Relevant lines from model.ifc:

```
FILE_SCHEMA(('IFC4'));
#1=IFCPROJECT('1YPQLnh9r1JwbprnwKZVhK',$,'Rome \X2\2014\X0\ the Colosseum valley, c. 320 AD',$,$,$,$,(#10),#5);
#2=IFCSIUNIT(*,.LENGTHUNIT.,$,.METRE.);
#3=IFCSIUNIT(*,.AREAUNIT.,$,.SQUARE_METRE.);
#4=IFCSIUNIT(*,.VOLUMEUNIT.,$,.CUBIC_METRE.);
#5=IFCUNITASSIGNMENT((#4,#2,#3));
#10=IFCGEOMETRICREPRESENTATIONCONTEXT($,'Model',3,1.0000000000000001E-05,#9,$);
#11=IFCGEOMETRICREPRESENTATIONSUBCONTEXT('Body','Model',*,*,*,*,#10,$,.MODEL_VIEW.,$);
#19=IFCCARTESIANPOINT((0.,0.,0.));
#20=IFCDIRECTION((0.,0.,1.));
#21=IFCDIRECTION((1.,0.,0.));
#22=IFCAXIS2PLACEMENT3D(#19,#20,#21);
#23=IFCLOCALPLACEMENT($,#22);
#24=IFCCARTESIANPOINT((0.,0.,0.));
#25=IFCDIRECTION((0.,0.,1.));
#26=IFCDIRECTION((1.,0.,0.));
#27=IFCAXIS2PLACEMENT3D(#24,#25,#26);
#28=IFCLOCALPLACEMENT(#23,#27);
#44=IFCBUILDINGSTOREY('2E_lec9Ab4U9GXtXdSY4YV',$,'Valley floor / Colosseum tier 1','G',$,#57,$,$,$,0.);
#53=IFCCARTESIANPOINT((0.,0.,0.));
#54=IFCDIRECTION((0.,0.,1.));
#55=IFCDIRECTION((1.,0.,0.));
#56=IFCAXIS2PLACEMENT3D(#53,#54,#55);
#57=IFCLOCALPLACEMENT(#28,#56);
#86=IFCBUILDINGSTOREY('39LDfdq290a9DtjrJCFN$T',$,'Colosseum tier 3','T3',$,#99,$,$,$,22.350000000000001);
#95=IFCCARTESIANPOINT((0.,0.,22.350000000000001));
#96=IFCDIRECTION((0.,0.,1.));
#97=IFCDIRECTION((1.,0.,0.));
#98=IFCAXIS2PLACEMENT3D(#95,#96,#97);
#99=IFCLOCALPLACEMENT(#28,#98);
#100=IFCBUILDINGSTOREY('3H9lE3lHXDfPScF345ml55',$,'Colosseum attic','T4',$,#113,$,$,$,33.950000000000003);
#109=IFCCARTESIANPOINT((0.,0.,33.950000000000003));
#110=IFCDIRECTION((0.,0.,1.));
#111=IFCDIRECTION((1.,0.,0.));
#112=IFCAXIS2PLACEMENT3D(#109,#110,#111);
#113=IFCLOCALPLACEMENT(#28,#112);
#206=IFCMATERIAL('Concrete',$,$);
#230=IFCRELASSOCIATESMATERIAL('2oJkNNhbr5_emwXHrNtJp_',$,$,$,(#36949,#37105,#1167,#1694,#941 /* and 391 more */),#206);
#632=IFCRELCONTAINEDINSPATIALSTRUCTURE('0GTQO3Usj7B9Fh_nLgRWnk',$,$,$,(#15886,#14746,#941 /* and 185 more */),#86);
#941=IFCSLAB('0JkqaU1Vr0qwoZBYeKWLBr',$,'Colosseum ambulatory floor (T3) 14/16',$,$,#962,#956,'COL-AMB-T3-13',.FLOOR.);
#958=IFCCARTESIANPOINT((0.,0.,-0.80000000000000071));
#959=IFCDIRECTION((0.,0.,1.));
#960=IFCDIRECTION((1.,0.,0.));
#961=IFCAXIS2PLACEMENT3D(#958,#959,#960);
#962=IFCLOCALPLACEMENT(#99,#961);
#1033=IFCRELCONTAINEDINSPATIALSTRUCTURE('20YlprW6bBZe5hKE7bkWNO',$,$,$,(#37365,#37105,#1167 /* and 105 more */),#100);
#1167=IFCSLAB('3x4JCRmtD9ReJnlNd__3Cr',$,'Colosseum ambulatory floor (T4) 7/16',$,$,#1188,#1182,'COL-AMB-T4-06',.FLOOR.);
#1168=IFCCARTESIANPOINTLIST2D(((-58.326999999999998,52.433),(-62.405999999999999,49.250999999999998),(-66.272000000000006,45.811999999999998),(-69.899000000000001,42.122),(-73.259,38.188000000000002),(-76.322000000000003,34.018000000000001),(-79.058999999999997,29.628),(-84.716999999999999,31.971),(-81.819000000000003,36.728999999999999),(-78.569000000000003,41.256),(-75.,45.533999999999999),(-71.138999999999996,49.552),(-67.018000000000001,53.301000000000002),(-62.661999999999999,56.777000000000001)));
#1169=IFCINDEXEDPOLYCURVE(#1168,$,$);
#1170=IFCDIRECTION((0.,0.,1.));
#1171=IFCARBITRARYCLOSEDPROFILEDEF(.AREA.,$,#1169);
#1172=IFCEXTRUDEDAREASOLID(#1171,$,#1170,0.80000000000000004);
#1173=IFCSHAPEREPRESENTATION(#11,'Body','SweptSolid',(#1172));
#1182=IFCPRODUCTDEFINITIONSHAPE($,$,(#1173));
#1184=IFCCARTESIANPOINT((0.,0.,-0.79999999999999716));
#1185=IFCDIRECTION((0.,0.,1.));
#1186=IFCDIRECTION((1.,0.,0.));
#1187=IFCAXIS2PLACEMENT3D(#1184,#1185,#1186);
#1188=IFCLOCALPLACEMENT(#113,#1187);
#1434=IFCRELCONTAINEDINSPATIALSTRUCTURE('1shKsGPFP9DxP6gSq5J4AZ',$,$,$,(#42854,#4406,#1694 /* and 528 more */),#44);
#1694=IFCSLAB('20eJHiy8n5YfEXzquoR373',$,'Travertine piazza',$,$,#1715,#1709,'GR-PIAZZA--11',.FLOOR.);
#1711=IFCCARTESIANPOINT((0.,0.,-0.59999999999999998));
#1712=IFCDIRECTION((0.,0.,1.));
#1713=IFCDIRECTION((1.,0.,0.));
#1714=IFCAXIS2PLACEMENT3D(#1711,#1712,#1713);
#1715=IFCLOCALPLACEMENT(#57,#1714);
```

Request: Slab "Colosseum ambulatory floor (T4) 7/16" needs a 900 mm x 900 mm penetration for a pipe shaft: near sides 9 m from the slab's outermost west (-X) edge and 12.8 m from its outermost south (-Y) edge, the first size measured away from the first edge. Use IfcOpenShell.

```python
import numpy as np
import ifcopenshell
import ifcopenshell.api.feature
import ifcopenshell.api.geometry
import ifcopenshell.api.root
import ifcopenshell.geom
import ifcopenshell.util.placement
import ifcopenshell.util.representation
import ifcopenshell.util.shape
import ifcopenshell.util.unit

model = ifcopenshell.open("model.ifc")
unit_scale = ifcopenshell.util.unit.calculate_unit_scale(model)
settings = ifcopenshell.geom.settings()


def volume(element):
    """Net volume in cubic metres, openings subtracted."""
    shape = ifcopenshell.geom.create_shape(settings, element)
    return ifcopenshell.util.shape.get_volume(shape.geometry)


slab = model.by_id(1167)
before = volume(slab)

# Extent in the slab's own axes, in metres. The edges named are its -X and -Y sides.
slab_shape = ifcopenshell.geom.create_shape(settings, slab)
vertices = ifcopenshell.util.shape.get_vertices(slab_shape.geometry)
x_min, y_min, bottom = vertices.min(axis=0)
top = vertices[:, 2].max()

opening = ifcopenshell.api.root.create_entity(model, ifc_class="IfcOpeningElement", name="Pipe shaft opening", predefined_type="OPENING")
context = ifcopenshell.util.representation.get_context(model, "Model", "Body", "MODEL_VIEW")
width, depth = 0.9, 0.9
outline = [(0.0, 0.0), (width, 0.0), (width, depth), (0.0, depth), (0.0, 0.0)]
# Overshoot both faces by 50 mm so the cut is clean.
shape = ifcopenshell.api.geometry.add_slab_representation(
    model, context=context, depth=top - bottom + 0.1, polyline=outline
)
ifcopenshell.api.geometry.assign_representation(model, product=opening, representation=shape)

matrix = ifcopenshell.util.placement.get_local_placement(slab.ObjectPlacement)
matrix[:, 3] = matrix @ np.append(np.array([x_min + 9, y_min + 12.8, bottom - 0.05]) / unit_scale, 1.0)
ifcopenshell.api.geometry.edit_object_placement(model, product=opening, matrix=matrix, is_si=False)
ifcopenshell.api.feature.add_feature(model, feature=opening, element=slab)

after = volume(slab)

print(f"slab volume {before:.3f} -> {after:.3f} m3")

model.write("model_edited.ifc")
```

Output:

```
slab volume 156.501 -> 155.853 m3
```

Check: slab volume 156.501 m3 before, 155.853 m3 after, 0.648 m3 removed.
